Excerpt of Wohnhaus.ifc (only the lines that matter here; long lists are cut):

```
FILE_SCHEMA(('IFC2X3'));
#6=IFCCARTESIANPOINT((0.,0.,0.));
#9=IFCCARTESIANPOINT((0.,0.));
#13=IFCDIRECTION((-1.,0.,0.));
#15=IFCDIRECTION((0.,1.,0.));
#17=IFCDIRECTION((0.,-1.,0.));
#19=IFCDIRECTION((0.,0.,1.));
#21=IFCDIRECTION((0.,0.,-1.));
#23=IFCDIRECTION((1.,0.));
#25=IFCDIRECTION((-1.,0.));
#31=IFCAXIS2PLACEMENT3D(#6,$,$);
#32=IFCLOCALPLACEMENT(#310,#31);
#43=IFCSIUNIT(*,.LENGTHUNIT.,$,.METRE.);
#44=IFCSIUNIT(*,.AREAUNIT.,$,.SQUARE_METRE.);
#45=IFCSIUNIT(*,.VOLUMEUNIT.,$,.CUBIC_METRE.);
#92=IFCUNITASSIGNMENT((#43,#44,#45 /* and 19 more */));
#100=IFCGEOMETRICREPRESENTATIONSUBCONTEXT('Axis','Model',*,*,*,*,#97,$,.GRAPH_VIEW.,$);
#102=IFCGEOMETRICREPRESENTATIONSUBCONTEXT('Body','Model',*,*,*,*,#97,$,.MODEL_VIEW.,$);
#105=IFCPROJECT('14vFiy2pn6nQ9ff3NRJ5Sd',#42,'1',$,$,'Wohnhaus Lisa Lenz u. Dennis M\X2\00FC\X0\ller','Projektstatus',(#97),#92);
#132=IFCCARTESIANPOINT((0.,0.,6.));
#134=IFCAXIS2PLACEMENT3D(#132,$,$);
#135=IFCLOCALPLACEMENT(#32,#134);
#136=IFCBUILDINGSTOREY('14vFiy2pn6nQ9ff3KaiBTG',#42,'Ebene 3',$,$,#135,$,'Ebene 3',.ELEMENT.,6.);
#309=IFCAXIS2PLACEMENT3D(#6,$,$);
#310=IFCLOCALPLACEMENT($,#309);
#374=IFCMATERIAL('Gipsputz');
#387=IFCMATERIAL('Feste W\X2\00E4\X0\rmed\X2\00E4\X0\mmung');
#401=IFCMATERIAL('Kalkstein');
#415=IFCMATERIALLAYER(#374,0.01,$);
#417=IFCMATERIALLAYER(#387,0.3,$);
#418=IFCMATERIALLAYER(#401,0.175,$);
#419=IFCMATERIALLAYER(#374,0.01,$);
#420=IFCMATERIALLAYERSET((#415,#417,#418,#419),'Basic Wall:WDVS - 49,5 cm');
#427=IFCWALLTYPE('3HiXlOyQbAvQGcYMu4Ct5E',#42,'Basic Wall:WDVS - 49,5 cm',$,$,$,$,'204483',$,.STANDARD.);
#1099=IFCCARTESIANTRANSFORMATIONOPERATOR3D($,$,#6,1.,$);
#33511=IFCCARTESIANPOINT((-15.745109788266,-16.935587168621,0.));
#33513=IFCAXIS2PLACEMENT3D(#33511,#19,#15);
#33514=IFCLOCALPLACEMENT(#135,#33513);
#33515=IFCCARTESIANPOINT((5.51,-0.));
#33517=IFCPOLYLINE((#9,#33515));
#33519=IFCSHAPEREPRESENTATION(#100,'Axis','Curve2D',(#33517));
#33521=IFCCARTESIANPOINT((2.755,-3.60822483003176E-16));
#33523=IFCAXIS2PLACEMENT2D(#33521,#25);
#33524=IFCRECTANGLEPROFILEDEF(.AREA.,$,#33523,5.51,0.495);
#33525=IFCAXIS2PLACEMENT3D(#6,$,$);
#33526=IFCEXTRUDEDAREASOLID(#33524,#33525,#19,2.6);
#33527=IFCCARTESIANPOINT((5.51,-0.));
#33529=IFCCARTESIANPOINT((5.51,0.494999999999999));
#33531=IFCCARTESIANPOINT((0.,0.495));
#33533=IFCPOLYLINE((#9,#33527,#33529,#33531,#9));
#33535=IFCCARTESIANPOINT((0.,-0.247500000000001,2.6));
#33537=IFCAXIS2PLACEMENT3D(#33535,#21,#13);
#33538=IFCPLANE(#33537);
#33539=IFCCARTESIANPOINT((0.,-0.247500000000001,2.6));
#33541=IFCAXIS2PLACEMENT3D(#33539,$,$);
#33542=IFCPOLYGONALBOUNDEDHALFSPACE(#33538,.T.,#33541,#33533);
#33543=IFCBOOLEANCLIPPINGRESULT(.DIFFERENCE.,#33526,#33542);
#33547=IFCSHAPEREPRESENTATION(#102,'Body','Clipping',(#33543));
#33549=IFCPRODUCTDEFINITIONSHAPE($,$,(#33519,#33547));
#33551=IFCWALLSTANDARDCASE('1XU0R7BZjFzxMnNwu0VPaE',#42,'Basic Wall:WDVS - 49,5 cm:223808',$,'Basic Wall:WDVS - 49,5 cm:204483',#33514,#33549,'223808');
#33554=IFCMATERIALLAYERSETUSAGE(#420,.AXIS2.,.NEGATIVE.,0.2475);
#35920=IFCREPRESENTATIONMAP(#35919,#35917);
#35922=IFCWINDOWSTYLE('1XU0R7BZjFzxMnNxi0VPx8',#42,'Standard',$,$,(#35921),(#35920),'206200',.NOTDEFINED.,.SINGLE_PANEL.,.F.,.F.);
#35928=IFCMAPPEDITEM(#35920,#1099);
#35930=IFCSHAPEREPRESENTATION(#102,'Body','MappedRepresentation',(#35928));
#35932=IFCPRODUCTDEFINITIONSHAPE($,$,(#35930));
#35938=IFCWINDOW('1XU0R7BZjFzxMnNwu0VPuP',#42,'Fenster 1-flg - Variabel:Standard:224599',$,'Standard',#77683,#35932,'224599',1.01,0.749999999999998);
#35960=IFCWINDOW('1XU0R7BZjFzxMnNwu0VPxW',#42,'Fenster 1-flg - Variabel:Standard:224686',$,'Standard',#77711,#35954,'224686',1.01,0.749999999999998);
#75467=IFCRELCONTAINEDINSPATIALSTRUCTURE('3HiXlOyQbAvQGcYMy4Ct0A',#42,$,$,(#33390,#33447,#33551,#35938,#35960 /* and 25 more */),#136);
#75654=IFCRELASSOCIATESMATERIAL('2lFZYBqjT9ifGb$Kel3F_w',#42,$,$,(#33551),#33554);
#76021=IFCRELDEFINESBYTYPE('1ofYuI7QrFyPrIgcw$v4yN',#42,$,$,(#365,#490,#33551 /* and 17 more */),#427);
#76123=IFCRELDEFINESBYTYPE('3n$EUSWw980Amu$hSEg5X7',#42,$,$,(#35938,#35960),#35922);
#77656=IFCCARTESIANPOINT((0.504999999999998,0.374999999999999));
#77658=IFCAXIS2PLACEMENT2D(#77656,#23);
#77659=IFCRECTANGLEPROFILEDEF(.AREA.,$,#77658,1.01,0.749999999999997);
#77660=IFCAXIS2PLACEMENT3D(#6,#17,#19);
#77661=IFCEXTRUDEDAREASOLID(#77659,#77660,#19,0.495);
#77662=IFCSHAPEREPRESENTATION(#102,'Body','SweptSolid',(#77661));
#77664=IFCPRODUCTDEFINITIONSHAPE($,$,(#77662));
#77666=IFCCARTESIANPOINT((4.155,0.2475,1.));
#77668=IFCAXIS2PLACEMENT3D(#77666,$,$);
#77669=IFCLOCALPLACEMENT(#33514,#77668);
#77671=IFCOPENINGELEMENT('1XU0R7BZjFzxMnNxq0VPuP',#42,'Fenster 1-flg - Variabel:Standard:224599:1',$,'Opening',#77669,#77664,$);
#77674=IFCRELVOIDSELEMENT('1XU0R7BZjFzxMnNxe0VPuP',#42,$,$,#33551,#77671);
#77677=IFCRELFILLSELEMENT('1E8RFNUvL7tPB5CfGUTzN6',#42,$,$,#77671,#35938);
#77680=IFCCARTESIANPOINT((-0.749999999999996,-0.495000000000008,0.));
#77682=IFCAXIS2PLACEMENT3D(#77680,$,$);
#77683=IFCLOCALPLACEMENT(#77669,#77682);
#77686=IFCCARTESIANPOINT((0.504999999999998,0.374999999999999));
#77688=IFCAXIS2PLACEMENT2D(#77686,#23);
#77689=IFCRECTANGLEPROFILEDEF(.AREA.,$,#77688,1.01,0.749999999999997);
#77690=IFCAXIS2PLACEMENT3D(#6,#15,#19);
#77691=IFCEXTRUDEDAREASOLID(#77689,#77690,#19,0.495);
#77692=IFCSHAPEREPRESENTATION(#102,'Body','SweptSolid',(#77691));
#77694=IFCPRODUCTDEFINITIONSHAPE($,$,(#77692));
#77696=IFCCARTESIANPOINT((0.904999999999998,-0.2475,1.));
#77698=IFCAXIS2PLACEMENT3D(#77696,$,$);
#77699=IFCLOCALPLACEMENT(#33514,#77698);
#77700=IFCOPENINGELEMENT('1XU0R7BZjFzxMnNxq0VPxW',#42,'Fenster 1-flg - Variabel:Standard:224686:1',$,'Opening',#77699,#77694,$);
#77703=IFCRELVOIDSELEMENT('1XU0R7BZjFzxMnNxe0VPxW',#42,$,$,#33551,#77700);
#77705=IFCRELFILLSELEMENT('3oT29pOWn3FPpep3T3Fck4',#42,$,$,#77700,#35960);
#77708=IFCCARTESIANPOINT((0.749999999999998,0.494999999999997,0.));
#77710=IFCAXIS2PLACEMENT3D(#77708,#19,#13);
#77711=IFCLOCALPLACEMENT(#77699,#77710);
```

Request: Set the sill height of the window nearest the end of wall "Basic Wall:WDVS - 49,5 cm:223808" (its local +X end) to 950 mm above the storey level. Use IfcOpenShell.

```python
import numpy as np
import ifcopenshell
import ifcopenshell.api.geometry
import ifcopenshell.geom
import ifcopenshell.util.element
import ifcopenshell.util.placement
import ifcopenshell.util.shape
import ifcopenshell.util.unit

model = ifcopenshell.open("Wohnhaus.ifc")
unit_scale = ifcopenshell.util.unit.calculate_unit_scale(model)

window = model.by_guid("1XU0R7BZjFzxMnNwu0VPuP")
opening = window.FillsVoids[0].RelatingOpeningElement
storey = ifcopenshell.util.element.get_container(window, ifc_class="IfcBuildingStorey")
level = ifcopenshell.util.placement.get_local_placement(storey.ObjectPlacement)[2, 3]

# The opening's origin need not be at the sill, so measure its lowest point.
shape = ifcopenshell.geom.create_shape(ifcopenshell.geom.settings(), opening)
bottom = ifcopenshell.util.shape.get_shape_bottom_elevation(shape, shape.geometry) / unit_scale
dz = level + 0.95 - bottom

shift = np.array([0.0, 0.0, dz])
# The window is placed relative to its opening, so it follows when the opening moves.
matrix = ifcopenshell.util.placement.get_local_placement(opening.ObjectPlacement)
matrix[:3, 3] += shift
ifcopenshell.api.geometry.edit_object_placement(
    model, product=opening, matrix=matrix, is_si=False, should_transform_children=True
)

print(f"moved by {dz * unit_scale:+.3f} m")

model.write("Wohnhaus_updated.ifc")
```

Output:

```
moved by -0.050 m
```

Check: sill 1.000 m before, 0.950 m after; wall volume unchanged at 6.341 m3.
